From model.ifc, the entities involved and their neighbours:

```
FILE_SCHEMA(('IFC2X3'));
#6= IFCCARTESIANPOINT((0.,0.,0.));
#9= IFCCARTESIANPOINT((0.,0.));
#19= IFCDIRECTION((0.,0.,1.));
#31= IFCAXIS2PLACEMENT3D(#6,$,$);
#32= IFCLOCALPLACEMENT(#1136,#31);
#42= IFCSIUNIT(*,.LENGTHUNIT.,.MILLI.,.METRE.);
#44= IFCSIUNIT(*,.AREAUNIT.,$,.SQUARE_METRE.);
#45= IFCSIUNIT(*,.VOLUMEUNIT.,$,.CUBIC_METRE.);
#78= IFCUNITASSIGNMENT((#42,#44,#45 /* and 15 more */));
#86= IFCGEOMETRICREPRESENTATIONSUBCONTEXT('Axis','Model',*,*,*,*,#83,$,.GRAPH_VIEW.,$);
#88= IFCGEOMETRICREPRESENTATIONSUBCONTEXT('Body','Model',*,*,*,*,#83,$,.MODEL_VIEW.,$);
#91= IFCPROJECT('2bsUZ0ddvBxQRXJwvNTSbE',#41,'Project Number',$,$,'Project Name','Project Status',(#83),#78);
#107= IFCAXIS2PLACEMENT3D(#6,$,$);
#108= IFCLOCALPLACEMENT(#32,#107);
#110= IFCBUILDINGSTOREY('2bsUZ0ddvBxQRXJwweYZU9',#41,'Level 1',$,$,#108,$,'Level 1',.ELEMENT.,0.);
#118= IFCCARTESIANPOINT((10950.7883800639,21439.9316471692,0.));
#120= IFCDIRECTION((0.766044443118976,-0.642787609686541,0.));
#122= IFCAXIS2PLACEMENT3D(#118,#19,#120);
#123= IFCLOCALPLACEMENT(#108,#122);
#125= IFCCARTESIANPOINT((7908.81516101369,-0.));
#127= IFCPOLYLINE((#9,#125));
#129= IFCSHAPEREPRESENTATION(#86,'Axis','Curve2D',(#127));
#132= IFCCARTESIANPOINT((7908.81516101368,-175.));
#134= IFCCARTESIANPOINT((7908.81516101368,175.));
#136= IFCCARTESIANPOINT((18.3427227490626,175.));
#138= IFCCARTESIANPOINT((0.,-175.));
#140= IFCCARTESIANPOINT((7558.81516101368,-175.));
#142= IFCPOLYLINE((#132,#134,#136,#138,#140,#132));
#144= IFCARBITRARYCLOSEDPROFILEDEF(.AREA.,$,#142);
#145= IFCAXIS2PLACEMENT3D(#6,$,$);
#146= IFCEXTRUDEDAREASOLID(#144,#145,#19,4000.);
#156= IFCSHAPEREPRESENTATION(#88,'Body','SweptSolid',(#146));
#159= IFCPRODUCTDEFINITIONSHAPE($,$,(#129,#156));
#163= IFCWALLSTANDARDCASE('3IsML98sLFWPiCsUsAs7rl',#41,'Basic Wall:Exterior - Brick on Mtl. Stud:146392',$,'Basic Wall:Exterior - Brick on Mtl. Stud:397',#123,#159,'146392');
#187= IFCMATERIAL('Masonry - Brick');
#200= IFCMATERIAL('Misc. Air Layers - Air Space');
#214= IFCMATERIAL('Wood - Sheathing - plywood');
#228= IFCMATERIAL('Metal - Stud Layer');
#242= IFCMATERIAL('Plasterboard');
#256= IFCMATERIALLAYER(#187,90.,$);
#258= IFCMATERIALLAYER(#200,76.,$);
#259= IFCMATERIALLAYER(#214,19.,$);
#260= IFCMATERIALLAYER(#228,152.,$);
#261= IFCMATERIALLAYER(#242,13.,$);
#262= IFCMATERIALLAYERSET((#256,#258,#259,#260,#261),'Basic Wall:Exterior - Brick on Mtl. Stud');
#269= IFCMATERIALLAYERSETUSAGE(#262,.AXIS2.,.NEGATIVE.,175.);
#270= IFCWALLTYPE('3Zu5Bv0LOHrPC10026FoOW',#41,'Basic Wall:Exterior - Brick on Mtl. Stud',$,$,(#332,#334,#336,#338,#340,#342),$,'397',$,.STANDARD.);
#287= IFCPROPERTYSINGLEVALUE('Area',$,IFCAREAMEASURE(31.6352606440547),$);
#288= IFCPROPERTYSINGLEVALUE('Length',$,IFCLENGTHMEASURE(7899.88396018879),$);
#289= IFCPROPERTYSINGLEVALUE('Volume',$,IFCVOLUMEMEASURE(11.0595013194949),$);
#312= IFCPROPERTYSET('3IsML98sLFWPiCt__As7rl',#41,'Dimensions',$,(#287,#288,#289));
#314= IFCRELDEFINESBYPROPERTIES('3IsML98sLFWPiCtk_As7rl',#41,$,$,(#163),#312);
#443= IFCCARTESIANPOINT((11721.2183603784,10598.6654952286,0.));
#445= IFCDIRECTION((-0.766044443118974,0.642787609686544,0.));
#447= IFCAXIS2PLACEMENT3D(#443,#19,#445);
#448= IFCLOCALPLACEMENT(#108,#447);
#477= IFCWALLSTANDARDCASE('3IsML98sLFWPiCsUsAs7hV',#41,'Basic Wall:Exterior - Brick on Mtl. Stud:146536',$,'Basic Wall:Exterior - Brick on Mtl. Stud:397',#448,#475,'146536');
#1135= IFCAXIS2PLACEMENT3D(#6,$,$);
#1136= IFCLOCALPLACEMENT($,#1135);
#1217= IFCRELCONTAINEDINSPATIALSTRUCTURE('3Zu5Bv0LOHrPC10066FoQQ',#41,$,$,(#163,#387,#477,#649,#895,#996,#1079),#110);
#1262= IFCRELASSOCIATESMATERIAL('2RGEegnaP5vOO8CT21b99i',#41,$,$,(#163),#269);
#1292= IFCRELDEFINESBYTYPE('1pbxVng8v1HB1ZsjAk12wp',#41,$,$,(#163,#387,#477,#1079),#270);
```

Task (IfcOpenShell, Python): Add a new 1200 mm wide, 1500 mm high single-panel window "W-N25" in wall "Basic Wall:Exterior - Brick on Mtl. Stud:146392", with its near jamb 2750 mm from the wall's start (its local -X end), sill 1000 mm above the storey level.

```python
import numpy as np
import ifcopenshell
import ifcopenshell.api.feature
import ifcopenshell.api.geometry
import ifcopenshell.api.pset
import ifcopenshell.api.root
import ifcopenshell.api.spatial
import ifcopenshell.api.type
import ifcopenshell.geom
import ifcopenshell.util.element
import ifcopenshell.util.placement
import ifcopenshell.util.representation
import ifcopenshell.util.shape
import ifcopenshell.util.unit

model = ifcopenshell.open("model.ifc")
unit_scale = ifcopenshell.util.unit.calculate_unit_scale(model)
area_scale = ifcopenshell.util.unit.calculate_unit_scale(model, "AREAUNIT")
volume_scale = ifcopenshell.util.unit.calculate_unit_scale(model, "VOLUMEUNIT")
settings = ifcopenshell.geom.settings()


def volume(element):
    """Net volume in cubic metres, openings subtracted."""
    shape = ifcopenshell.geom.create_shape(settings, element)
    return ifcopenshell.util.shape.get_volume(shape.geometry)


wall = model.by_guid("3IsML98sLFWPiCsUsAs7rl")
storey = ifcopenshell.util.element.get_container(wall, ifc_class="IfcBuildingStorey")
context = ifcopenshell.util.representation.get_context(model, "Model", "Body", "MODEL_VIEW")
before = volume(wall)

width, height, from_end, sill = 1.2, 1.5, 2.75, 1  # metres

# The wall runs along its own X axis, and the end named is its -X end.
wall_shape = ifcopenshell.geom.create_shape(settings, wall)
x, y, z = ifcopenshell.util.shape.get_vertices(wall_shape.geometry).T
start = x.min() + from_end
face, thickness = float(y.min()), float(y.max() - y.min())
wall_matrix = ifcopenshell.util.placement.get_local_placement(wall.ObjectPlacement)
level = ifcopenshell.util.placement.get_local_placement(storey.ObjectPlacement)[2, 3]


def in_wall(x, y):
    """Placement at x, y metres in the wall's axes, at sill height."""
    matrix = wall_matrix.copy()
    matrix[:, 3] = wall_matrix @ np.array([x / unit_scale, y / unit_scale, 0.0, 1.0])
    matrix[2, 3] = level + sill / unit_scale
    return matrix


# Opening: a box that overshoots both wall faces by 50 mm.
opening = ifcopenshell.api.root.create_entity(model, ifc_class="IfcOpeningElement")
box = ifcopenshell.api.geometry.add_wall_representation(
    model, context=context, length=width, height=height, thickness=thickness + 0.1
)
ifcopenshell.api.geometry.assign_representation(model, product=opening, representation=box)
ifcopenshell.api.geometry.edit_object_placement(model, product=opening, matrix=in_wall(start, face - 0.05), is_si=False)
ifcopenshell.api.feature.add_feature(model, feature=opening, element=wall)

window = ifcopenshell.api.root.create_entity(model, ifc_class="IfcWindow", name="W-N25")
window.OverallWidth, window.OverallHeight = width / unit_scale, height / unit_scale
body = ifcopenshell.api.geometry.add_window_representation(
    model,
    context=context,
    overall_width=window.OverallWidth,
    overall_height=window.OverallHeight,
    partition_type="SINGLE_PANEL",
)
ifcopenshell.api.geometry.assign_representation(model, product=window, representation=body)
ifcopenshell.api.spatial.assign_container(model, products=[window], relating_structure=storey)
fills = ifcopenshell.api.feature.add_filling(model, opening=opening, element=window)
fills.OwnerHistory = window.OwnerHistory  # required in IFC2X3

# IFC2X3 keeps the operation on the window style.
style = ifcopenshell.api.root.create_entity(model, ifc_class="IfcWindowStyle", name="W-N25")
style.OperationType, style.ConstructionType = "SINGLE_PANEL", "NOTDEFINED"
style.ParameterTakesPrecedence = style.Sizeable = False
ifcopenshell.api.type.assign_type(model, related_objects=[window], relating_type=style)

# Centre the window in the wall's thickness.
ifcopenshell.api.geometry.edit_object_placement(model, product=window, matrix=in_wall(start, face), is_si=False)
window_shape = ifcopenshell.geom.create_shape(settings, window)
depth = ifcopenshell.util.shape.get_vertices(window_shape.geometry)[:, 1]
offset = face + thickness / 2 - (depth.min() + depth.max()) / 2
ifcopenshell.api.geometry.edit_object_placement(model, product=window, matrix=in_wall(start, offset), is_si=False)

after = volume(wall)

# Update the wall's stored quantities.
pset = model.by_id(ifcopenshell.util.element.get_pset(wall, "Dimensions", should_inherit=False)["id"])
ifcopenshell.api.pset.edit_pset(model, pset=pset, properties={
    "Area": model.create_entity("IfcAreaMeasure", after / thickness / area_scale),
    "Volume": model.create_entity("IfcVolumeMeasure", after / volume_scale),
})

print(f"wall volume {before:.3f} -> {after:.3f} m3")

model.write("model_updated.ifc")
```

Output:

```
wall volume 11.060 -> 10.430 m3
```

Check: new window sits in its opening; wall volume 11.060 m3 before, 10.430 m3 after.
